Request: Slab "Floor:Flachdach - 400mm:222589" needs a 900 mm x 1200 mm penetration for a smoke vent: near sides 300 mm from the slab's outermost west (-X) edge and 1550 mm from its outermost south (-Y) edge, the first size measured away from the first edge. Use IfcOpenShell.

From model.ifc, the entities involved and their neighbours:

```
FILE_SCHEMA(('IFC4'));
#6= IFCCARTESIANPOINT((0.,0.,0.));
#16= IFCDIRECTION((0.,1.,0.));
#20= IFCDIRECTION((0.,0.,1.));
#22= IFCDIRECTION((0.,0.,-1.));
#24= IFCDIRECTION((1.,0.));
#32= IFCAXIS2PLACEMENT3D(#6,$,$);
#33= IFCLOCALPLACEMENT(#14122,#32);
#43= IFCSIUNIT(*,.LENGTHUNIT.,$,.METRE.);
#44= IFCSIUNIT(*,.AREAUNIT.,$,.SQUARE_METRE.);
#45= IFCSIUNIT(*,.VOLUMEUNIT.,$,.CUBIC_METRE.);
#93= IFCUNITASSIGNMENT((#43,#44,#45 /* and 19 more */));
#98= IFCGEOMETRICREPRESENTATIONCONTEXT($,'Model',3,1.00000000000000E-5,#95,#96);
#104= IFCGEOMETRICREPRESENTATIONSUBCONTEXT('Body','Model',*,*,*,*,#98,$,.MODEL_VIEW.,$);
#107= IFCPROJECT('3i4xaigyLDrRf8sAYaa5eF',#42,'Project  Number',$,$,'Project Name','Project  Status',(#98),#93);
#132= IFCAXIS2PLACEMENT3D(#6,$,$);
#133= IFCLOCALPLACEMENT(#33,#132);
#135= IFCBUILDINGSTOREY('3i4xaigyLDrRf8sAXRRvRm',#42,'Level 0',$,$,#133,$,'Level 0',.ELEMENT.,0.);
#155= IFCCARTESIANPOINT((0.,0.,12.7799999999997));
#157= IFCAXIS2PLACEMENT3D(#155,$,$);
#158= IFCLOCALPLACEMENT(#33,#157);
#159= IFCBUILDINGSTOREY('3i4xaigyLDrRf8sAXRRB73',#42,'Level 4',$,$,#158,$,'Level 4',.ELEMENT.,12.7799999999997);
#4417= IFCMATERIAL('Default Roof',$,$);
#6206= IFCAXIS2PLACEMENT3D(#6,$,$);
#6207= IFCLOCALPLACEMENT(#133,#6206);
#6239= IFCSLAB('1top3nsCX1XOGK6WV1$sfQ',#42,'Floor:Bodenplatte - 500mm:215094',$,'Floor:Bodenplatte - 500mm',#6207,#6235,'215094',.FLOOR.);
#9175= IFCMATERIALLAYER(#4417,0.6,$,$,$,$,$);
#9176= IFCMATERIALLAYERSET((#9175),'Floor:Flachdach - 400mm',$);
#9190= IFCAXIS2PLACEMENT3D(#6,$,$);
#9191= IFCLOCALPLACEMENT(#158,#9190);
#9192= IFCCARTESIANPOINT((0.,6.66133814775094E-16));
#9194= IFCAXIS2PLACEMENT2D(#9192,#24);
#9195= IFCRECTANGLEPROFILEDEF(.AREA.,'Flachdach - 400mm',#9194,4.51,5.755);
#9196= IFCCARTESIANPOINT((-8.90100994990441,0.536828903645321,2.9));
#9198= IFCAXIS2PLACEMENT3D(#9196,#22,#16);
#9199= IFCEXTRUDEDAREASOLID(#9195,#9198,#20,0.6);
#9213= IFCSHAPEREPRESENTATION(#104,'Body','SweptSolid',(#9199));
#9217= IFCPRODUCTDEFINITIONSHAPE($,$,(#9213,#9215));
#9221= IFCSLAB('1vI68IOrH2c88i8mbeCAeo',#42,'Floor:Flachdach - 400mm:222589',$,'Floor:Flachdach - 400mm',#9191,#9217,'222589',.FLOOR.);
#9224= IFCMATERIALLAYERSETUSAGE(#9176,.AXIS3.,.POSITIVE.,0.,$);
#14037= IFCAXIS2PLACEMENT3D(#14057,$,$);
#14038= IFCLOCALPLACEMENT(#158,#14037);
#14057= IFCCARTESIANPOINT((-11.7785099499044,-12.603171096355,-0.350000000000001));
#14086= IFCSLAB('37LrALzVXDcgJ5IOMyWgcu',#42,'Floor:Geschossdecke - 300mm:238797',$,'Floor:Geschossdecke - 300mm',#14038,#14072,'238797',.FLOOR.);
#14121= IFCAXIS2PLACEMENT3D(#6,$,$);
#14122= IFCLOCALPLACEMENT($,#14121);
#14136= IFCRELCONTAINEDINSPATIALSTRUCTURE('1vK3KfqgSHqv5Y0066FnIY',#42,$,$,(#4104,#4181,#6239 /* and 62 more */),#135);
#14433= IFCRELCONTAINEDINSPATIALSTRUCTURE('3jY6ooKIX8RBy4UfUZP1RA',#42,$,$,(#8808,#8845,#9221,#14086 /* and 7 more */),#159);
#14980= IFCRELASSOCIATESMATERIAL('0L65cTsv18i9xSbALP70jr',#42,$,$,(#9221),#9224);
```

```python
import numpy as np
import ifcopenshell
import ifcopenshell.api.feature
import ifcopenshell.api.geometry
import ifcopenshell.api.root
import ifcopenshell.geom
import ifcopenshell.util.placement
import ifcopenshell.util.representation
import ifcopenshell.util.shape
import ifcopenshell.util.unit

model = ifcopenshell.open("model.ifc")
unit_scale = ifcopenshell.util.unit.calculate_unit_scale(model)
settings = ifcopenshell.geom.settings()


def volume(element):
    """Net volume in cubic metres, openings subtracted."""
    shape = ifcopenshell.geom.create_shape(settings, element)
    return ifcopenshell.util.shape.get_volume(shape.geometry)


slab = model.by_guid("1vI68IOrH2c88i8mbeCAeo")
before = volume(slab)

# Extent in the slab's own axes, in metres. The edges named are its -X and -Y sides.
slab_shape = ifcopenshell.geom.create_shape(settings, slab)
vertices = ifcopenshell.util.shape.get_vertices(slab_shape.geometry)
x_min, y_min, bottom = vertices.min(axis=0)
top = vertices[:, 2].max()

opening = ifcopenshell.api.root.create_entity(model, ifc_class="IfcOpeningElement", name="Smoke vent opening", predefined_type="OPENING")
context = ifcopenshell.util.representation.get_context(model, "Model", "Body", "MODEL_VIEW")
width, depth = 0.9, 1.2
outline = [(0.0, 0.0), (width, 0.0), (width, depth), (0.0, depth), (0.0, 0.0)]
# Overshoot both faces by 50 mm so the cut is clean.
shape = ifcopenshell.api.geometry.add_slab_representation(
    model, context=context, depth=top - bottom + 0.1, polyline=outline
)
ifcopenshell.api.geometry.assign_representation(model, product=opening, representation=shape)

matrix = ifcopenshell.util.placement.get_local_placement(slab.ObjectPlacement)
matrix[:, 3] = matrix @ np.append(np.array([x_min + 0.3, y_min + 1.55, bottom - 0.05]) / unit_scale, 1.0)
ifcopenshell.api.geometry.edit_object_placement(model, product=opening, matrix=matrix, is_si=False)
ifcopenshell.api.feature.add_feature(model, feature=opening, element=slab)

after = volume(slab)

print(f"slab volume {before:.3f} -> {after:.3f} m3")

model.write("model_v2.ifc")
```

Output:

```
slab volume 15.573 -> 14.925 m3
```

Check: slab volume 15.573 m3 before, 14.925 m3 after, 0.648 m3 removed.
